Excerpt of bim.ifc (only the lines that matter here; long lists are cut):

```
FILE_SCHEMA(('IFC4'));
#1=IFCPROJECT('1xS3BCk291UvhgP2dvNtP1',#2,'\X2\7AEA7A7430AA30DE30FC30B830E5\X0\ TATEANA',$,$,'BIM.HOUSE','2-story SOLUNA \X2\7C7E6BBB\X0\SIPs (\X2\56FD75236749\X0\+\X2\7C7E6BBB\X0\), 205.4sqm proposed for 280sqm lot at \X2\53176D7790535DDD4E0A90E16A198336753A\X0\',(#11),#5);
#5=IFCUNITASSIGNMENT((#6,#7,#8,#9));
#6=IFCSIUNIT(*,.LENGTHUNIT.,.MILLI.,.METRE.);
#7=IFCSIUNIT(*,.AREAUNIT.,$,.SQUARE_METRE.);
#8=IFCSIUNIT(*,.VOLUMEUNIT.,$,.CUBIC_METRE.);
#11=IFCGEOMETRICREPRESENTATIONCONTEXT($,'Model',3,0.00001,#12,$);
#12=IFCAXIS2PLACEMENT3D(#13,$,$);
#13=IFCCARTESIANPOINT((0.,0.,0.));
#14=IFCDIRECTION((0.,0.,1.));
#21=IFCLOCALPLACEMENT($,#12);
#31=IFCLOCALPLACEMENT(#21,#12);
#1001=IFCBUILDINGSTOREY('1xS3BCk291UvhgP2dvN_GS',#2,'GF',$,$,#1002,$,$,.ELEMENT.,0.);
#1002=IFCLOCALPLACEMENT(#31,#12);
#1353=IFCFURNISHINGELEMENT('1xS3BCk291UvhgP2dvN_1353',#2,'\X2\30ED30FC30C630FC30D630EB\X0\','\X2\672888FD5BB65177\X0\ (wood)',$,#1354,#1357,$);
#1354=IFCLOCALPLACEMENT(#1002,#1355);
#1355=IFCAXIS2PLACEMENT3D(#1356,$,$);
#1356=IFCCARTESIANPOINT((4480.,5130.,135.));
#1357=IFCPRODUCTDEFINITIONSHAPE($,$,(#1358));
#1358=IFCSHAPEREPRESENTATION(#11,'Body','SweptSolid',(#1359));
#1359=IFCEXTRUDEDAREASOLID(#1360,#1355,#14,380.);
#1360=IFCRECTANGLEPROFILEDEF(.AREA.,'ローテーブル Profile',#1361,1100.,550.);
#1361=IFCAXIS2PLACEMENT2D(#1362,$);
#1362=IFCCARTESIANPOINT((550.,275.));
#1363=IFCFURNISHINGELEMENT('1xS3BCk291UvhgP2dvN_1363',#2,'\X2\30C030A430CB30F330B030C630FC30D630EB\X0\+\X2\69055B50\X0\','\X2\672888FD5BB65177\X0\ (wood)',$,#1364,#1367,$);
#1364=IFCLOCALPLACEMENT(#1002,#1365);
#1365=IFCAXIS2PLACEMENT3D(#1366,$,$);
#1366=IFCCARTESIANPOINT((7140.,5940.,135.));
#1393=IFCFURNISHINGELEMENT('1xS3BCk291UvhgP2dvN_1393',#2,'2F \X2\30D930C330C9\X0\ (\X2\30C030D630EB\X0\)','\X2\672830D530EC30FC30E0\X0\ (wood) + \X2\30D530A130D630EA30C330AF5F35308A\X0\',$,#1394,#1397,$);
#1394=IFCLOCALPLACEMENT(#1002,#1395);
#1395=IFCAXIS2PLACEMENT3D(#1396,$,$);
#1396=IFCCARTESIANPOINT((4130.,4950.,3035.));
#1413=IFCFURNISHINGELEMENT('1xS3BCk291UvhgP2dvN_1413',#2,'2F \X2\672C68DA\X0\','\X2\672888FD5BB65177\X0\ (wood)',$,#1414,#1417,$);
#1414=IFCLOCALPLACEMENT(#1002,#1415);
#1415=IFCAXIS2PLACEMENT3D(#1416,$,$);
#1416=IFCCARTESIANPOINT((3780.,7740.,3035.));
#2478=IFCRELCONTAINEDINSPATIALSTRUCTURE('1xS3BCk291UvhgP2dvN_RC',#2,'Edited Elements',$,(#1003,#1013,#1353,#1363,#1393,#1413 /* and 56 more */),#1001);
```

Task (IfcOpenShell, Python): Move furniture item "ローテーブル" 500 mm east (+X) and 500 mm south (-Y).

```python
import ifcopenshell
import ifcopenshell.api.geometry
import ifcopenshell.util.placement
import ifcopenshell.util.unit

model = ifcopenshell.open("bim.ifc")
unit_scale = ifcopenshell.util.unit.calculate_unit_scale(model)

item = model.by_guid("1xS3BCk291UvhgP2dvN_1353")
matrix = ifcopenshell.util.placement.get_local_placement(item.ObjectPlacement)
matrix[0, 3] += 0.5 / unit_scale
matrix[1, 3] -= 0.5 / unit_scale
ifcopenshell.api.geometry.edit_object_placement(model, product=item, matrix=matrix, is_si=False)

print(ifcopenshell.util.placement.get_local_placement(item.ObjectPlacement).round(3) + 0.0)

model.write("bim_updated.ifc")
```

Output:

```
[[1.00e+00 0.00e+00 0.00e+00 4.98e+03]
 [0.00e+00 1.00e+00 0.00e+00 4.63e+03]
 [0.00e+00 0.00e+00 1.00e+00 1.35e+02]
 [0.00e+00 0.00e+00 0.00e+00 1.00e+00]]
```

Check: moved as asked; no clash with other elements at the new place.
